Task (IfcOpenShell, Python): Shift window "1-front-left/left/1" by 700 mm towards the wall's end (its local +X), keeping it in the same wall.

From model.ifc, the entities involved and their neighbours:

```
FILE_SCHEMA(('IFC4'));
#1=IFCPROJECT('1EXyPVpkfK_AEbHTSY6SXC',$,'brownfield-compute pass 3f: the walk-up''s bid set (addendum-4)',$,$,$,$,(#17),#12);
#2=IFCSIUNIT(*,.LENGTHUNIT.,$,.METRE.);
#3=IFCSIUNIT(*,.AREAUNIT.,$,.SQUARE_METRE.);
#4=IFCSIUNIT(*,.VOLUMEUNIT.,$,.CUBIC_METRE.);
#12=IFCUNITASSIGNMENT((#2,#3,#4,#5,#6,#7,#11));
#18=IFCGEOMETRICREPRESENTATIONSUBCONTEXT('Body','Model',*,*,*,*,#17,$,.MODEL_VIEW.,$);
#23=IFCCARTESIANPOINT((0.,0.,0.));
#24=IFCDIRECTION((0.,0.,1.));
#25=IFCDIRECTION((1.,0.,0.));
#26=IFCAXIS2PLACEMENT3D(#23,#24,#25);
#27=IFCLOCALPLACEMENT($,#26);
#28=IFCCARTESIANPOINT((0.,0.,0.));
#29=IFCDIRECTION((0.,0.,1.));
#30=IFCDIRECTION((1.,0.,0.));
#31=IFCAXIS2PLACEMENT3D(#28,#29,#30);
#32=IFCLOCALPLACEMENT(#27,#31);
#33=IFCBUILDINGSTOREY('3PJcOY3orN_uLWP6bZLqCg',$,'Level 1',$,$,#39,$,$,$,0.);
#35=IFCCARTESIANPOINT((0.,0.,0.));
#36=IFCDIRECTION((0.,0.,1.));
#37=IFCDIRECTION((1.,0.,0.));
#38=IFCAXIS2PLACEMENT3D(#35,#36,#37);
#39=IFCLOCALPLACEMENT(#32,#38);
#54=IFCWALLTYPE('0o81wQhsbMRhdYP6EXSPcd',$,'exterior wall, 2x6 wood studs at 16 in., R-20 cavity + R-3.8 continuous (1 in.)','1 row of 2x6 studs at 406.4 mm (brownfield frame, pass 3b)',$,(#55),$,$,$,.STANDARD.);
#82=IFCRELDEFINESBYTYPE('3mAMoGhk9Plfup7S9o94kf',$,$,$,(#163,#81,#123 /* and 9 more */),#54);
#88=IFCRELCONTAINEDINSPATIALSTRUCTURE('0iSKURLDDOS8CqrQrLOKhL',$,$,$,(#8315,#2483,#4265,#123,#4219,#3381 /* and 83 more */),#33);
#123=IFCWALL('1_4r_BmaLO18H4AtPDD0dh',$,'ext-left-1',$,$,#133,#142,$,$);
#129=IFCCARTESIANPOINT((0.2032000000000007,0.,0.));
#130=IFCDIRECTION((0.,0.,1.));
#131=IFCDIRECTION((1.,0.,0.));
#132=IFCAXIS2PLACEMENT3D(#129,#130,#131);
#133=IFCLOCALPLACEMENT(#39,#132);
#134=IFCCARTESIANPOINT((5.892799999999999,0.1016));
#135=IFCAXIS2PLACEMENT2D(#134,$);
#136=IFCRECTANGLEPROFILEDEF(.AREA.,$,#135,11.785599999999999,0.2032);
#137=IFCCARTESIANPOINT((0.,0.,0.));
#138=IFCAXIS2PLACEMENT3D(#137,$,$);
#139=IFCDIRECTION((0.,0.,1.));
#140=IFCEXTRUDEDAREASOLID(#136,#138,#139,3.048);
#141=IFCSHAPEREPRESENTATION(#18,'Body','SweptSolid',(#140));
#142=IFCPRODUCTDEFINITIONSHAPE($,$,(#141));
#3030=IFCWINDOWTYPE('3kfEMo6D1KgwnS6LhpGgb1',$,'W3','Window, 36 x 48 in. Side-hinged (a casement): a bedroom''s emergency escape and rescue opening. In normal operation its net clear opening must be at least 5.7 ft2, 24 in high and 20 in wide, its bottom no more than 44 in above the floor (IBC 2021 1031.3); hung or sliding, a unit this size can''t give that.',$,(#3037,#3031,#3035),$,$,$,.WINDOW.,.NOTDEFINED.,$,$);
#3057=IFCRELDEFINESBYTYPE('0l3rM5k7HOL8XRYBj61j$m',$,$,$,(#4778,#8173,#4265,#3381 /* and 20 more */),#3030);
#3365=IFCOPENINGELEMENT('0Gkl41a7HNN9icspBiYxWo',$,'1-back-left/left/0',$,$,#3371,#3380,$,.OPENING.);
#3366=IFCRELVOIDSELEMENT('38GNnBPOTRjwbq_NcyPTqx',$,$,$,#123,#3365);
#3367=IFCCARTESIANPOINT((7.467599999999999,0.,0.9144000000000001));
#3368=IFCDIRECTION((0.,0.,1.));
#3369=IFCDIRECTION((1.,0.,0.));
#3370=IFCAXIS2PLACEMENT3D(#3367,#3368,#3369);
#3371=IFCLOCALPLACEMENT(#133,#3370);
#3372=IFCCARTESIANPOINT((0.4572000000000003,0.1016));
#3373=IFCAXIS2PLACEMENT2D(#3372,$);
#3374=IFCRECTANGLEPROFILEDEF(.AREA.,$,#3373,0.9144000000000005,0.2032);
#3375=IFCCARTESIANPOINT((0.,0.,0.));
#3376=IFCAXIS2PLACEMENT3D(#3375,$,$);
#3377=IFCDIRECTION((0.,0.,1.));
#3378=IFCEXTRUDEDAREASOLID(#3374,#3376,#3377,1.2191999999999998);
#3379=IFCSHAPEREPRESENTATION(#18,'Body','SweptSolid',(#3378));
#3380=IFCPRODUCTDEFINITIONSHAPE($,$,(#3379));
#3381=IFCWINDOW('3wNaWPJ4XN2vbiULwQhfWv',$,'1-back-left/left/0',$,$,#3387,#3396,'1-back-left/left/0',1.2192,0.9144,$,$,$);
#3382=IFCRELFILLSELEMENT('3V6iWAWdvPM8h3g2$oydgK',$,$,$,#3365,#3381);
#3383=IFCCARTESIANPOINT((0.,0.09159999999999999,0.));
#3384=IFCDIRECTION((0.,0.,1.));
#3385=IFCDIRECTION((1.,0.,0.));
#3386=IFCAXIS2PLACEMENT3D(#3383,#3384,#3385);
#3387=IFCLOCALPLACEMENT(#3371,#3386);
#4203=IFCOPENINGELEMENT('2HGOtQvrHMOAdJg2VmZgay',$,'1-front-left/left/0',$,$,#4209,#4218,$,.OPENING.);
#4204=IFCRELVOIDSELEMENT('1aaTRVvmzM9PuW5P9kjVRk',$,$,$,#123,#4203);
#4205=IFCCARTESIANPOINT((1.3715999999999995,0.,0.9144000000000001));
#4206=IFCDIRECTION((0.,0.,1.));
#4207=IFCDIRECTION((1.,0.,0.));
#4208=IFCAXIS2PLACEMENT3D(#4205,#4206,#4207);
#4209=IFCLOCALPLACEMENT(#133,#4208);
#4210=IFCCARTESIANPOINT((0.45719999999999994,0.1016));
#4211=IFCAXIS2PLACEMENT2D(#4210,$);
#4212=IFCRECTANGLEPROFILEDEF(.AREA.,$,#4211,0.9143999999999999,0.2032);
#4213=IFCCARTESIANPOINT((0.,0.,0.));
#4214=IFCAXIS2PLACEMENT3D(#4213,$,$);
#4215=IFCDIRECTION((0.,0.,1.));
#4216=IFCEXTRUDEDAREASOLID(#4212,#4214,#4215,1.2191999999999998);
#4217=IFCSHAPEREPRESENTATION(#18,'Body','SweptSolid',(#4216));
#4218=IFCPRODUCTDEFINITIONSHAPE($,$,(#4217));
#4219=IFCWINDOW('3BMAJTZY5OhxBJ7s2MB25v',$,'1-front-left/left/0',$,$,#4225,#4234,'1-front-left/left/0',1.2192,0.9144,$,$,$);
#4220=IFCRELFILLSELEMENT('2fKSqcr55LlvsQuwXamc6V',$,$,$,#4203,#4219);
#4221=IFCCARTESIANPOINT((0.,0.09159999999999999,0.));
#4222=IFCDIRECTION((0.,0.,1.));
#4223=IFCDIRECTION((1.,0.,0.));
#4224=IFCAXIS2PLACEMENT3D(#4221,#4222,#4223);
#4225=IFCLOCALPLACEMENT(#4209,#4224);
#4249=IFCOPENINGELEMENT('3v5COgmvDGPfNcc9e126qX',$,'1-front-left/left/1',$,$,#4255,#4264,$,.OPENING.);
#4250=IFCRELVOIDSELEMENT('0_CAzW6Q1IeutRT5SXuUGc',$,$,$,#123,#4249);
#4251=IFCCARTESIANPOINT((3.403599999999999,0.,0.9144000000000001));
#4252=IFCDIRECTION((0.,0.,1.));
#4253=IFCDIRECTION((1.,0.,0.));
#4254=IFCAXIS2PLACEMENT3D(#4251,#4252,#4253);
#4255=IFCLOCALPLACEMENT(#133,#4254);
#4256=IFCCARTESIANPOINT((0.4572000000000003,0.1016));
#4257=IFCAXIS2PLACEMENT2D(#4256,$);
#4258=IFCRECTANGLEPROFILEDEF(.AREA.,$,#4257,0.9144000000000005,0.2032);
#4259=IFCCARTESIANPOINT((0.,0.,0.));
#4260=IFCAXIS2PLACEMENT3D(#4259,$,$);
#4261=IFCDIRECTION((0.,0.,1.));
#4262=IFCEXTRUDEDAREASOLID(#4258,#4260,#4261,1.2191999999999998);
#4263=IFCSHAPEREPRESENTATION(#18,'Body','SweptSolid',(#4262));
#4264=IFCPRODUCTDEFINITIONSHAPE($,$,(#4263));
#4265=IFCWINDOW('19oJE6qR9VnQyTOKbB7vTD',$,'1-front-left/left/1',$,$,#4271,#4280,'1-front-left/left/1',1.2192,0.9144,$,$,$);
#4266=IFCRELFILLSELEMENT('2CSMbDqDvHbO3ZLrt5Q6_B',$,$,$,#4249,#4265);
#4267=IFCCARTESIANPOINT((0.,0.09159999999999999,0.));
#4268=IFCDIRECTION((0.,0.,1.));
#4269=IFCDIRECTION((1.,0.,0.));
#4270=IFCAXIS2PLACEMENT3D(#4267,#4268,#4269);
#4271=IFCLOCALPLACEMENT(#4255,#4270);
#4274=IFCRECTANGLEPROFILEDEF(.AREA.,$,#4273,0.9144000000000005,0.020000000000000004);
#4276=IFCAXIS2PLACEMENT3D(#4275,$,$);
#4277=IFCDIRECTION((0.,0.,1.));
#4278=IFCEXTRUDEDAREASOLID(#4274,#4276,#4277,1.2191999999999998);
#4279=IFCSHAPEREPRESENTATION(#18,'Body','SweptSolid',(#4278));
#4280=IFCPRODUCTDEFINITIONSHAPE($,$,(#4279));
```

```python
import ifcopenshell
import ifcopenshell.api.geometry
import ifcopenshell.util.placement

model = ifcopenshell.open("model.ifc")

window = model.by_guid("19oJE6qR9VnQyTOKbB7vTD")
opening = window.FillsVoids[0].RelatingOpeningElement
wall = opening.VoidsElements[0].RelatingBuildingElement

wall_matrix = ifcopenshell.util.placement.get_local_placement(wall.ObjectPlacement)
shift = wall_matrix[:3, 0] * 0.7
before = ifcopenshell.util.placement.get_local_placement(window.ObjectPlacement)[:3, 3].copy()

# The window is placed relative to its opening, so it follows when the opening moves.
matrix = ifcopenshell.util.placement.get_local_placement(opening.ObjectPlacement)
matrix[:3, 3] += shift
ifcopenshell.api.geometry.edit_object_placement(
    model, product=opening, matrix=matrix, is_si=False, should_transform_children=True
)

after = ifcopenshell.util.placement.get_local_placement(window.ObjectPlacement)[:3, 3]
print("window moved by", (after - before).round(3) + 0.0)

model.write("model-out.ifc")
```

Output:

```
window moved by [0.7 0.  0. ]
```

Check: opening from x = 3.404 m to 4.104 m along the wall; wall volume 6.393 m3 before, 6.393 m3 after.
